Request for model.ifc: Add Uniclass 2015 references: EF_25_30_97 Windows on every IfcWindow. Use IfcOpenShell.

First a look at what the model holds.

```python
import ifcopenshell

model = ifcopenshell.open("model.ifc")
print(model.schema)
print("classifications:", [c.Name for c in model.by_type("IfcClassification")])
for ifc_class in ("IfcDoor", "IfcRoof", "IfcStair", "IfcWall", "IfcWindow"):
    print(ifc_class, len(model.by_type(ifc_class)))
```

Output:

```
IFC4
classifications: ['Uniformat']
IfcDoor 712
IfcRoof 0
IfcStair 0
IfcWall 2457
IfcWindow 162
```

```python
import ifcopenshell
import ifcopenshell.api.classification

model = ifcopenshell.open("model.ifc")

system = ifcopenshell.api.classification.add_classification(model, classification="Uniclass 2015")

codes = {
    "IfcWindow": ("EF_25_30_97", "Windows"),
}
for ifc_class, (code, name) in codes.items():
    products = model.by_type(ifc_class)
    ifcopenshell.api.classification.add_reference(
        model, products=products, classification=system, identification=code, name=name
    )
    print(code, len(products))

model.write("model-out.ifc")
```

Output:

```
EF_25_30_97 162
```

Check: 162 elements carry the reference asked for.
